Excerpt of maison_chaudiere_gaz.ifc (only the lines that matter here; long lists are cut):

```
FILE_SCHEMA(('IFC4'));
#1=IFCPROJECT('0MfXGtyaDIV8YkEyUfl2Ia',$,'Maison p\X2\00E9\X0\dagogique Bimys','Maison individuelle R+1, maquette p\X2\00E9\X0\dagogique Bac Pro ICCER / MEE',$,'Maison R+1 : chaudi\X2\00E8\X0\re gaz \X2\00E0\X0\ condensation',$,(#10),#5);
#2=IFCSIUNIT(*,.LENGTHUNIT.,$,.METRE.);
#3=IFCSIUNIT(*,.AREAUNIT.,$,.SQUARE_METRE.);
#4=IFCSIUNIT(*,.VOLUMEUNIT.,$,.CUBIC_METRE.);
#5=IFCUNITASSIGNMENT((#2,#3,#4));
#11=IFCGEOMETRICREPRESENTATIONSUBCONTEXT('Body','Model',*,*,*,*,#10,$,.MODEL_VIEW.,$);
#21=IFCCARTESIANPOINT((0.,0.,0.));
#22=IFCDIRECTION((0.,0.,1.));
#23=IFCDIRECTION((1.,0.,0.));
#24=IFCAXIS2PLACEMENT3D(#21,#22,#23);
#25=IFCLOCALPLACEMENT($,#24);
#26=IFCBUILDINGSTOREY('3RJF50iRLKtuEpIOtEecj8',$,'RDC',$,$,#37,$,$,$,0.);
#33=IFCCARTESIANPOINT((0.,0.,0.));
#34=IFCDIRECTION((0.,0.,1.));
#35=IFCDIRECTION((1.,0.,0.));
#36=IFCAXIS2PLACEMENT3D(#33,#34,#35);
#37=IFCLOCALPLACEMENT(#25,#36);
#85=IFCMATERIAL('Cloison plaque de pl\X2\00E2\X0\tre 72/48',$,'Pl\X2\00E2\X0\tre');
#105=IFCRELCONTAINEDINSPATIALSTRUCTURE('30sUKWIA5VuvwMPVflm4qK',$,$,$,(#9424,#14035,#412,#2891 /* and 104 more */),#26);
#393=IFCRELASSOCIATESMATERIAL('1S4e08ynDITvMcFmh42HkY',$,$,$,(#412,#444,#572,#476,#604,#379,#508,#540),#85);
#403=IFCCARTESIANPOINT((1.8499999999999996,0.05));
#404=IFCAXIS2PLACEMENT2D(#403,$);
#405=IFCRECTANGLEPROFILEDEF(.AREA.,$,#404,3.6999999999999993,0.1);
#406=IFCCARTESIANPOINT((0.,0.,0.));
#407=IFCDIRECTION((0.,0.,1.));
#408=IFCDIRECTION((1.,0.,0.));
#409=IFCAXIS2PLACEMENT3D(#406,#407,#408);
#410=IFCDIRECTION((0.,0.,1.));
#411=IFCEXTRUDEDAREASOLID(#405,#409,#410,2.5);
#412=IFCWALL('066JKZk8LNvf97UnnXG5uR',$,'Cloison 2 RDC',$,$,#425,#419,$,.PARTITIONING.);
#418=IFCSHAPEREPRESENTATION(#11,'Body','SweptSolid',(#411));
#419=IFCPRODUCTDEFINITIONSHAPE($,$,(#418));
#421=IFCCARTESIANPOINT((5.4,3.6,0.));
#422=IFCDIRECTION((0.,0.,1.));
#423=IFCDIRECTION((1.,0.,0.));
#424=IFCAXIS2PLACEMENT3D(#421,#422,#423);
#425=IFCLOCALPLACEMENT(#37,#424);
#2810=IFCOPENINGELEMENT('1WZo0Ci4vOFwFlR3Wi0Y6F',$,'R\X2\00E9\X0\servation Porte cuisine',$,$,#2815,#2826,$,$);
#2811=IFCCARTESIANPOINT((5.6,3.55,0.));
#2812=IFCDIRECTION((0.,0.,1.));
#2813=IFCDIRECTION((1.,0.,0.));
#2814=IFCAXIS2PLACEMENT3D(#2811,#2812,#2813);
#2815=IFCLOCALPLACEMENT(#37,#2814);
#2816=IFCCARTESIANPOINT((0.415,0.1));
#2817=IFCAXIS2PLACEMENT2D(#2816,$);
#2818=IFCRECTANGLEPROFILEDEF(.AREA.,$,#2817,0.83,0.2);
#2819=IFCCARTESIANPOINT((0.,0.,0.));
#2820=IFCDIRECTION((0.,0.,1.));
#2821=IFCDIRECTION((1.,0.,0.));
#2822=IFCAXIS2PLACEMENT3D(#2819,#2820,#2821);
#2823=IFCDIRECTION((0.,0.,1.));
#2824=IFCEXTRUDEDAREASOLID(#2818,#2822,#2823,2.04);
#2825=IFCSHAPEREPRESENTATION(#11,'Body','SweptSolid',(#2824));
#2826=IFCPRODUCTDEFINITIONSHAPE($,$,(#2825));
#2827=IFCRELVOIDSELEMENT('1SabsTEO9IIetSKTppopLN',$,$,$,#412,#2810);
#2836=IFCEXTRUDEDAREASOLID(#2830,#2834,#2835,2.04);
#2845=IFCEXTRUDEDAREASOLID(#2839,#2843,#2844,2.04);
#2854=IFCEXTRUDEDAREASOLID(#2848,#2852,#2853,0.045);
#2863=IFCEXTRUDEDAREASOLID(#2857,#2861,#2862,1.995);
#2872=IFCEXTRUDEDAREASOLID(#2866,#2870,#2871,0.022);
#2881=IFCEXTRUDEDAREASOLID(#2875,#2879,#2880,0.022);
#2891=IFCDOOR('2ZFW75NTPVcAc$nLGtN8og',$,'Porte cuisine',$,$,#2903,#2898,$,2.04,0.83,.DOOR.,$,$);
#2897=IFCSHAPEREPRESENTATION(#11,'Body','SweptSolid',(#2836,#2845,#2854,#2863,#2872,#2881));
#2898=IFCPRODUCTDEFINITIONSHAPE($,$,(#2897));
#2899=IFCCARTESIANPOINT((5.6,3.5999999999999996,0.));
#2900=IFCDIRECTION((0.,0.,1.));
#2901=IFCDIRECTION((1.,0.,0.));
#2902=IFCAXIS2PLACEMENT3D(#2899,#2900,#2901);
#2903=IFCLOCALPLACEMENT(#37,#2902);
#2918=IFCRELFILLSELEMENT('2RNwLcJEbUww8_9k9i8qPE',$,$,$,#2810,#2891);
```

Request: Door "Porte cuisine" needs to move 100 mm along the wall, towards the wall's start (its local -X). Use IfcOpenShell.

```python
import ifcopenshell
import ifcopenshell.api.geometry
import ifcopenshell.util.placement

model = ifcopenshell.open("maison_chaudiere_gaz.ifc")

door = model.by_guid("2ZFW75NTPVcAc$nLGtN8og")
opening = door.FillsVoids[0].RelatingOpeningElement
wall = opening.VoidsElements[0].RelatingBuildingElement

wall_matrix = ifcopenshell.util.placement.get_local_placement(wall.ObjectPlacement)
shift = wall_matrix[:3, 0] * -0.1
before = ifcopenshell.util.placement.get_local_placement(door.ObjectPlacement)[:3, 3].copy()

# The door is not placed relative to its opening, so move both.
for product in (opening, door):
    matrix = ifcopenshell.util.placement.get_local_placement(product.ObjectPlacement)
    matrix[:3, 3] += shift
    ifcopenshell.api.geometry.edit_object_placement(model, product=product, matrix=matrix, is_si=False)

after = ifcopenshell.util.placement.get_local_placement(door.ObjectPlacement)[:3, 3]
print("door moved by", (after - before).round(3) + 0.0)

model.write("maison_chaudiere_gaz_v2.ifc")
```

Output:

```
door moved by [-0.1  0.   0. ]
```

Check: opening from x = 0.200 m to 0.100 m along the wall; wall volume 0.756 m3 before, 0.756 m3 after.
